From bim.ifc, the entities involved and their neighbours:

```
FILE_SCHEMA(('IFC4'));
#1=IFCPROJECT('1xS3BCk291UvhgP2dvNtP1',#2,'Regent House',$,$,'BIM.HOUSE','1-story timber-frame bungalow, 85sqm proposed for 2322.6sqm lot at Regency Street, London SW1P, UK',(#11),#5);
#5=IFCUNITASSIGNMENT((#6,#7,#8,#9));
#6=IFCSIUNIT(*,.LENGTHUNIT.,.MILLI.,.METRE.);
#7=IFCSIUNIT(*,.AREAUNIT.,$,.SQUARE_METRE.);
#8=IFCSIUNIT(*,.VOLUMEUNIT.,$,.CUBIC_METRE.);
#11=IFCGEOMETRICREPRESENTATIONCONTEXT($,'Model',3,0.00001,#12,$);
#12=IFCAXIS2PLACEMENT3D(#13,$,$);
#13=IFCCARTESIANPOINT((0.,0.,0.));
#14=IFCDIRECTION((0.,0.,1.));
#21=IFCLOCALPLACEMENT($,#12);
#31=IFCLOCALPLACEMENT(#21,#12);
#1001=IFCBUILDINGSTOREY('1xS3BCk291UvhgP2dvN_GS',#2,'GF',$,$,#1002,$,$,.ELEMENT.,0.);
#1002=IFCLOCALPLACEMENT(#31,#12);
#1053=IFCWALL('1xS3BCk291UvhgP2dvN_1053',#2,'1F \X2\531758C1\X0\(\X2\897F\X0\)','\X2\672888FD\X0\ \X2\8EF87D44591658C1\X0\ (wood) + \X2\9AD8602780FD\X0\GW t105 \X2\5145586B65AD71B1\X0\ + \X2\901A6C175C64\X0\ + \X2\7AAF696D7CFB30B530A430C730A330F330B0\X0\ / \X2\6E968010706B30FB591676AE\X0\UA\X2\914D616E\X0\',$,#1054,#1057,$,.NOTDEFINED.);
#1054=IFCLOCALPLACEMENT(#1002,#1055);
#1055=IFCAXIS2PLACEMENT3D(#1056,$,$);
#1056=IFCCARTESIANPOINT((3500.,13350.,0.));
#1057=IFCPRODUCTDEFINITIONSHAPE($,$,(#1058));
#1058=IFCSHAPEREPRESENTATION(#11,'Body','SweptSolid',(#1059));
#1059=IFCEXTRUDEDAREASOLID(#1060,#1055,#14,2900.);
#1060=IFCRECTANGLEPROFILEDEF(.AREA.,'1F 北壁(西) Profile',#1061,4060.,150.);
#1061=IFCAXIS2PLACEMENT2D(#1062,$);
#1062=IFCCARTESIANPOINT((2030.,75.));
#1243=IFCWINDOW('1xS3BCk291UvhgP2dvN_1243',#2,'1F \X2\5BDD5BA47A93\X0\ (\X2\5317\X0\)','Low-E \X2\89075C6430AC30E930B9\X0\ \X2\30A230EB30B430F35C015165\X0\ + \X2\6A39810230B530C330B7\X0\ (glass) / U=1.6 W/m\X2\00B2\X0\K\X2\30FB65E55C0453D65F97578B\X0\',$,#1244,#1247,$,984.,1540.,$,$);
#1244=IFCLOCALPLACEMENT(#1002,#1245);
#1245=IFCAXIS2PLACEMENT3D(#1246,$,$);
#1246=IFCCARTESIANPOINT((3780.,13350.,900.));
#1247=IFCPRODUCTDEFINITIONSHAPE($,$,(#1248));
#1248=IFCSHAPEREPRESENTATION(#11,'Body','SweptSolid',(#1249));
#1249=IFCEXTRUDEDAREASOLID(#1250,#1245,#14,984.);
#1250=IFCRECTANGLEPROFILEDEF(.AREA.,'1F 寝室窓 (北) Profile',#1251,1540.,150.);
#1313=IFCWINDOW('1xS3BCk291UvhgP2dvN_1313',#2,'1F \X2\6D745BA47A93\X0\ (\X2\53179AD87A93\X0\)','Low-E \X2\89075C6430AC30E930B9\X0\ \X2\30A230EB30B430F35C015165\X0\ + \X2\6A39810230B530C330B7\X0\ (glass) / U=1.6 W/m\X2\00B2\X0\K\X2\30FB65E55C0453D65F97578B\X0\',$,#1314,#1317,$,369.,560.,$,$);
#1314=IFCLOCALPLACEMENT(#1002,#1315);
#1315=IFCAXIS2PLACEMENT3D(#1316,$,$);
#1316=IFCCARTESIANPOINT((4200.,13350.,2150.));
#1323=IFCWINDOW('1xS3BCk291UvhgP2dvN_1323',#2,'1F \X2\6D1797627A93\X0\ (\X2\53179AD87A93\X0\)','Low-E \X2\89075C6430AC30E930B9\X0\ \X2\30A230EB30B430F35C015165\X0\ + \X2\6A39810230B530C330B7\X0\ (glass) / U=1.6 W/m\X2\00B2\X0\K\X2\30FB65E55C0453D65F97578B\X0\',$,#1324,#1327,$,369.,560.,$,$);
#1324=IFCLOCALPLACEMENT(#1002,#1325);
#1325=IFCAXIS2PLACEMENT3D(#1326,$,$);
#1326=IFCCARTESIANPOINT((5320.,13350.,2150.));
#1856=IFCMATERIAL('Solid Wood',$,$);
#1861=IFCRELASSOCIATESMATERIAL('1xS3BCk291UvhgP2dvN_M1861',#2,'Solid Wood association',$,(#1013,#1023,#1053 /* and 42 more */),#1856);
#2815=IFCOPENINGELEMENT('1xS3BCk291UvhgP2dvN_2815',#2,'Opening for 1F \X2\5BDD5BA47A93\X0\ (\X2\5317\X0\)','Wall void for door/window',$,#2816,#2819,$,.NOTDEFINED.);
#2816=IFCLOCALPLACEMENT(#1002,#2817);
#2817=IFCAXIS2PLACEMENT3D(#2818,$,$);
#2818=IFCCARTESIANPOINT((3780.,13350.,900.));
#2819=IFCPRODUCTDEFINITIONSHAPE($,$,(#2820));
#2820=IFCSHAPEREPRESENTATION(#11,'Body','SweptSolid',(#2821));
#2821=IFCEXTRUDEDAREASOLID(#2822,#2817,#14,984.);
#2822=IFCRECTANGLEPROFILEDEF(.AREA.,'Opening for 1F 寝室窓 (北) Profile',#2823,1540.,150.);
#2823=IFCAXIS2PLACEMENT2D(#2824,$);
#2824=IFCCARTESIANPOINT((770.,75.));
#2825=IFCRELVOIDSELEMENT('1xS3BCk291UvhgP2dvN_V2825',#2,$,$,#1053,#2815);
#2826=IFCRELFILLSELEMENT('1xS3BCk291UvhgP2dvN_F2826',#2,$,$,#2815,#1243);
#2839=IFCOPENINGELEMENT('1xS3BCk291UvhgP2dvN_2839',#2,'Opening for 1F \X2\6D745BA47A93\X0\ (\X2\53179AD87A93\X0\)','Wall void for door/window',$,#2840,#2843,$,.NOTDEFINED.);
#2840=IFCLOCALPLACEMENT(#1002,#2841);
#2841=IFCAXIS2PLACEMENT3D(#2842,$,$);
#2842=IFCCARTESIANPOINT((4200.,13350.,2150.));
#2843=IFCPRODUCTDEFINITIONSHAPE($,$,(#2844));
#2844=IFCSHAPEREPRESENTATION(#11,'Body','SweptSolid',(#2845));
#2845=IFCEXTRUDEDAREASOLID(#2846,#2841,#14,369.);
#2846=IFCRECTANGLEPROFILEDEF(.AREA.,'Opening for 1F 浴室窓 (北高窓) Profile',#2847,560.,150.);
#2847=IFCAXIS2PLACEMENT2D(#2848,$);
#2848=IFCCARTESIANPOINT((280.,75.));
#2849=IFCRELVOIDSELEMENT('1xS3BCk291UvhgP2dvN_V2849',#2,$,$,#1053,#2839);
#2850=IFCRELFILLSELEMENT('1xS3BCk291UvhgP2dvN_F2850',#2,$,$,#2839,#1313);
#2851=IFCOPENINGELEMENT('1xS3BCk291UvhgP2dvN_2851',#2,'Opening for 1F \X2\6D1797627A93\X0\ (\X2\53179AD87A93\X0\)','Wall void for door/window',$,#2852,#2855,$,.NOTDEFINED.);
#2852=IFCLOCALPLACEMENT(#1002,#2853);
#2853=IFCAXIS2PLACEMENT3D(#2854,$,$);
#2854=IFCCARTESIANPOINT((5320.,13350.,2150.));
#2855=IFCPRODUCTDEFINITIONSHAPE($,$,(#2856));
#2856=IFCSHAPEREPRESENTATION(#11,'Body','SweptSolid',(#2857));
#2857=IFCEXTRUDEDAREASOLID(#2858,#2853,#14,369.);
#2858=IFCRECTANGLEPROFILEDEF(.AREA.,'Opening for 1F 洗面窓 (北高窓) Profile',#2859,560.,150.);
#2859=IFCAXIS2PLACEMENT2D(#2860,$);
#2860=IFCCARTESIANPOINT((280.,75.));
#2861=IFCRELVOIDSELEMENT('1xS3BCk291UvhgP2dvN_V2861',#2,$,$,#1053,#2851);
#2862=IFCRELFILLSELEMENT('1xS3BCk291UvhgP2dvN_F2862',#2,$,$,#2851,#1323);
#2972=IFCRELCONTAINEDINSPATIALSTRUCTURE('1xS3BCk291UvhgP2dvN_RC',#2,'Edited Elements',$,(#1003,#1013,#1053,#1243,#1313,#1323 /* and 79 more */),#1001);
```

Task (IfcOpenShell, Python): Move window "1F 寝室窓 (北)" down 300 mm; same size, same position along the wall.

```python
import numpy as np
import ifcopenshell
import ifcopenshell.api.geometry
import ifcopenshell.util.placement
import ifcopenshell.util.unit

model = ifcopenshell.open("bim.ifc")
unit_scale = ifcopenshell.util.unit.calculate_unit_scale(model)

window = model.by_guid("1xS3BCk291UvhgP2dvN_1243")
opening = window.FillsVoids[0].RelatingOpeningElement
dz = -0.3 / unit_scale

shift = np.array([0.0, 0.0, dz])
# The window is not placed relative to its opening, so move both.
for product in (opening, window):
    matrix = ifcopenshell.util.placement.get_local_placement(product.ObjectPlacement)
    matrix[:3, 3] += shift
    ifcopenshell.api.geometry.edit_object_placement(model, product=product, matrix=matrix, is_si=False)

print(f"moved by {dz * unit_scale:+.3f} m")

model.write("bim_updated.ifc")
```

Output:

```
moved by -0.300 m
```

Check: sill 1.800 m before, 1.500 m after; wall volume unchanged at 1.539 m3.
